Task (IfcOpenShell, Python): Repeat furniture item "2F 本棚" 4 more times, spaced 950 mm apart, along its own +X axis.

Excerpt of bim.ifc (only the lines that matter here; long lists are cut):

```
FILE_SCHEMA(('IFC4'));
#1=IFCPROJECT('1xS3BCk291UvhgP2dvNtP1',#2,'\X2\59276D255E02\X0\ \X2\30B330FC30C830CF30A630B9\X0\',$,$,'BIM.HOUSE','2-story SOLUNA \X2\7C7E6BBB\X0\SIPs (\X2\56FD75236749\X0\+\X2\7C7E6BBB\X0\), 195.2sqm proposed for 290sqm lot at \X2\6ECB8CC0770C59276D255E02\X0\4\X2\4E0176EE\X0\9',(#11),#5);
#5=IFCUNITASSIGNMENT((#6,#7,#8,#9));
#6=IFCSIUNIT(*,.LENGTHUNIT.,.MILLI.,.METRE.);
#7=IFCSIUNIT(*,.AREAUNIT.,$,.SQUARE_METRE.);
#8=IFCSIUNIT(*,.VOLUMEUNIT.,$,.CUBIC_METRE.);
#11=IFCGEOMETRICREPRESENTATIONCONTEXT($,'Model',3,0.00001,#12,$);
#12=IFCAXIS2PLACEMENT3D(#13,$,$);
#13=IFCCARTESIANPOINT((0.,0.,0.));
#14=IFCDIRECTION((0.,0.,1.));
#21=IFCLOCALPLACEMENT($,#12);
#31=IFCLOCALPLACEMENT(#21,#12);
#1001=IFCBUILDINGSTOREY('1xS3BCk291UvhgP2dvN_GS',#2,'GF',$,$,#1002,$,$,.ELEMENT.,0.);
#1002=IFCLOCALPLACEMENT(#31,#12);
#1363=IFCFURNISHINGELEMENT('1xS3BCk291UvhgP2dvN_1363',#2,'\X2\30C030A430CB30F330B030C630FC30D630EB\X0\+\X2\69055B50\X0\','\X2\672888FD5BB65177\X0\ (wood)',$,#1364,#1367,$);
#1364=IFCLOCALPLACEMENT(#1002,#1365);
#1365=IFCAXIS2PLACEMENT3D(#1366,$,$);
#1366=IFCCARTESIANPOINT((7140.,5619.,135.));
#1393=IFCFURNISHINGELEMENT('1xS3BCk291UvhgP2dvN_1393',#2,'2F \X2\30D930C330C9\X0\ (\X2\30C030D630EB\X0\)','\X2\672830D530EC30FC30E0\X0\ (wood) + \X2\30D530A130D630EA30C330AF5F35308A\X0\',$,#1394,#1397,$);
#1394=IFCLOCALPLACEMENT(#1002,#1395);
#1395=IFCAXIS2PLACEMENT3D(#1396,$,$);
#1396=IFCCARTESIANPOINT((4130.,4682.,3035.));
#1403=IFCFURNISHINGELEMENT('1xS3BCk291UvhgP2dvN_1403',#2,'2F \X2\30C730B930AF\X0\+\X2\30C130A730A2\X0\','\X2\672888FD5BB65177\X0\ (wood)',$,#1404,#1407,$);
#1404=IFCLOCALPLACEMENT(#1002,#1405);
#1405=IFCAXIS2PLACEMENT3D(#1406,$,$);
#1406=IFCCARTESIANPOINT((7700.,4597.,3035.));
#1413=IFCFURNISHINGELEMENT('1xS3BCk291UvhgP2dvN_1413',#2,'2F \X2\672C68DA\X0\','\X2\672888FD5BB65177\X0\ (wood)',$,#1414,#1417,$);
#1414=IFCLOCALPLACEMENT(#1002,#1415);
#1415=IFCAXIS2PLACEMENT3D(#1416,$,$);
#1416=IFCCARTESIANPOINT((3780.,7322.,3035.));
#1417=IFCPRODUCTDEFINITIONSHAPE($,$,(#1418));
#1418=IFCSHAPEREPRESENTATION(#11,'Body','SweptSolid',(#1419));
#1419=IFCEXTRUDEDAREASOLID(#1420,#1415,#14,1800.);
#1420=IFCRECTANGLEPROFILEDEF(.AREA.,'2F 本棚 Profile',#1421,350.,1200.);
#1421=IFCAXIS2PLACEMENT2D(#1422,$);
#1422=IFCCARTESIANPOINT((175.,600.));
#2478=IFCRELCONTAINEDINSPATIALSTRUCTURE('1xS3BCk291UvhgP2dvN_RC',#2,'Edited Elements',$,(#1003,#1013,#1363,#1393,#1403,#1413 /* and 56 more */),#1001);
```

```python
import ifcopenshell
import ifcopenshell.api.geometry
import ifcopenshell.api.root
import ifcopenshell.util.element
import ifcopenshell.util.placement
import ifcopenshell.util.unit

model = ifcopenshell.open("bim.ifc")
unit_scale = ifcopenshell.util.unit.calculate_unit_scale(model)


def reuse_history(source, copy):
    """copy_class also copies each property set's owner history, people and application; keep the originals."""
    for rel in copy.IsDefinedBy:
        if rel.is_a("IfcRelDefinesByProperties") and (history := rel.RelatingPropertyDefinition.OwnerHistory):
            rel.RelatingPropertyDefinition.OwnerHistory = source.OwnerHistory
            ifcopenshell.util.element.remove_deep2(model, history)


source = model.by_guid("1xS3BCk291UvhgP2dvN_1413")
base = ifcopenshell.util.placement.get_local_placement(source.ObjectPlacement)
step = base[:3, 0] * 0.95 / unit_scale

for i in range(1, 5):
    copy = ifcopenshell.api.root.copy_class(model, product=source)
    copy.Representation = ifcopenshell.util.element.copy_deep(
        model, source.Representation, exclude=["IfcGeometricRepresentationContext", "IfcRepresentationMap"]
    )
    reuse_history(source, copy)
    matrix = base.copy()
    matrix[:3, 3] += i * step
    print("added at", matrix[:3, 3].round(3) + 0.0)
    ifcopenshell.api.geometry.edit_object_placement(model, product=copy, matrix=matrix, is_si=False)

model.write("bim_v2.ifc")
```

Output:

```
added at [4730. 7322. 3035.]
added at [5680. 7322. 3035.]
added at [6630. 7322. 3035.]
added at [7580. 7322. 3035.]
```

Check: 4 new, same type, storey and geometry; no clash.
